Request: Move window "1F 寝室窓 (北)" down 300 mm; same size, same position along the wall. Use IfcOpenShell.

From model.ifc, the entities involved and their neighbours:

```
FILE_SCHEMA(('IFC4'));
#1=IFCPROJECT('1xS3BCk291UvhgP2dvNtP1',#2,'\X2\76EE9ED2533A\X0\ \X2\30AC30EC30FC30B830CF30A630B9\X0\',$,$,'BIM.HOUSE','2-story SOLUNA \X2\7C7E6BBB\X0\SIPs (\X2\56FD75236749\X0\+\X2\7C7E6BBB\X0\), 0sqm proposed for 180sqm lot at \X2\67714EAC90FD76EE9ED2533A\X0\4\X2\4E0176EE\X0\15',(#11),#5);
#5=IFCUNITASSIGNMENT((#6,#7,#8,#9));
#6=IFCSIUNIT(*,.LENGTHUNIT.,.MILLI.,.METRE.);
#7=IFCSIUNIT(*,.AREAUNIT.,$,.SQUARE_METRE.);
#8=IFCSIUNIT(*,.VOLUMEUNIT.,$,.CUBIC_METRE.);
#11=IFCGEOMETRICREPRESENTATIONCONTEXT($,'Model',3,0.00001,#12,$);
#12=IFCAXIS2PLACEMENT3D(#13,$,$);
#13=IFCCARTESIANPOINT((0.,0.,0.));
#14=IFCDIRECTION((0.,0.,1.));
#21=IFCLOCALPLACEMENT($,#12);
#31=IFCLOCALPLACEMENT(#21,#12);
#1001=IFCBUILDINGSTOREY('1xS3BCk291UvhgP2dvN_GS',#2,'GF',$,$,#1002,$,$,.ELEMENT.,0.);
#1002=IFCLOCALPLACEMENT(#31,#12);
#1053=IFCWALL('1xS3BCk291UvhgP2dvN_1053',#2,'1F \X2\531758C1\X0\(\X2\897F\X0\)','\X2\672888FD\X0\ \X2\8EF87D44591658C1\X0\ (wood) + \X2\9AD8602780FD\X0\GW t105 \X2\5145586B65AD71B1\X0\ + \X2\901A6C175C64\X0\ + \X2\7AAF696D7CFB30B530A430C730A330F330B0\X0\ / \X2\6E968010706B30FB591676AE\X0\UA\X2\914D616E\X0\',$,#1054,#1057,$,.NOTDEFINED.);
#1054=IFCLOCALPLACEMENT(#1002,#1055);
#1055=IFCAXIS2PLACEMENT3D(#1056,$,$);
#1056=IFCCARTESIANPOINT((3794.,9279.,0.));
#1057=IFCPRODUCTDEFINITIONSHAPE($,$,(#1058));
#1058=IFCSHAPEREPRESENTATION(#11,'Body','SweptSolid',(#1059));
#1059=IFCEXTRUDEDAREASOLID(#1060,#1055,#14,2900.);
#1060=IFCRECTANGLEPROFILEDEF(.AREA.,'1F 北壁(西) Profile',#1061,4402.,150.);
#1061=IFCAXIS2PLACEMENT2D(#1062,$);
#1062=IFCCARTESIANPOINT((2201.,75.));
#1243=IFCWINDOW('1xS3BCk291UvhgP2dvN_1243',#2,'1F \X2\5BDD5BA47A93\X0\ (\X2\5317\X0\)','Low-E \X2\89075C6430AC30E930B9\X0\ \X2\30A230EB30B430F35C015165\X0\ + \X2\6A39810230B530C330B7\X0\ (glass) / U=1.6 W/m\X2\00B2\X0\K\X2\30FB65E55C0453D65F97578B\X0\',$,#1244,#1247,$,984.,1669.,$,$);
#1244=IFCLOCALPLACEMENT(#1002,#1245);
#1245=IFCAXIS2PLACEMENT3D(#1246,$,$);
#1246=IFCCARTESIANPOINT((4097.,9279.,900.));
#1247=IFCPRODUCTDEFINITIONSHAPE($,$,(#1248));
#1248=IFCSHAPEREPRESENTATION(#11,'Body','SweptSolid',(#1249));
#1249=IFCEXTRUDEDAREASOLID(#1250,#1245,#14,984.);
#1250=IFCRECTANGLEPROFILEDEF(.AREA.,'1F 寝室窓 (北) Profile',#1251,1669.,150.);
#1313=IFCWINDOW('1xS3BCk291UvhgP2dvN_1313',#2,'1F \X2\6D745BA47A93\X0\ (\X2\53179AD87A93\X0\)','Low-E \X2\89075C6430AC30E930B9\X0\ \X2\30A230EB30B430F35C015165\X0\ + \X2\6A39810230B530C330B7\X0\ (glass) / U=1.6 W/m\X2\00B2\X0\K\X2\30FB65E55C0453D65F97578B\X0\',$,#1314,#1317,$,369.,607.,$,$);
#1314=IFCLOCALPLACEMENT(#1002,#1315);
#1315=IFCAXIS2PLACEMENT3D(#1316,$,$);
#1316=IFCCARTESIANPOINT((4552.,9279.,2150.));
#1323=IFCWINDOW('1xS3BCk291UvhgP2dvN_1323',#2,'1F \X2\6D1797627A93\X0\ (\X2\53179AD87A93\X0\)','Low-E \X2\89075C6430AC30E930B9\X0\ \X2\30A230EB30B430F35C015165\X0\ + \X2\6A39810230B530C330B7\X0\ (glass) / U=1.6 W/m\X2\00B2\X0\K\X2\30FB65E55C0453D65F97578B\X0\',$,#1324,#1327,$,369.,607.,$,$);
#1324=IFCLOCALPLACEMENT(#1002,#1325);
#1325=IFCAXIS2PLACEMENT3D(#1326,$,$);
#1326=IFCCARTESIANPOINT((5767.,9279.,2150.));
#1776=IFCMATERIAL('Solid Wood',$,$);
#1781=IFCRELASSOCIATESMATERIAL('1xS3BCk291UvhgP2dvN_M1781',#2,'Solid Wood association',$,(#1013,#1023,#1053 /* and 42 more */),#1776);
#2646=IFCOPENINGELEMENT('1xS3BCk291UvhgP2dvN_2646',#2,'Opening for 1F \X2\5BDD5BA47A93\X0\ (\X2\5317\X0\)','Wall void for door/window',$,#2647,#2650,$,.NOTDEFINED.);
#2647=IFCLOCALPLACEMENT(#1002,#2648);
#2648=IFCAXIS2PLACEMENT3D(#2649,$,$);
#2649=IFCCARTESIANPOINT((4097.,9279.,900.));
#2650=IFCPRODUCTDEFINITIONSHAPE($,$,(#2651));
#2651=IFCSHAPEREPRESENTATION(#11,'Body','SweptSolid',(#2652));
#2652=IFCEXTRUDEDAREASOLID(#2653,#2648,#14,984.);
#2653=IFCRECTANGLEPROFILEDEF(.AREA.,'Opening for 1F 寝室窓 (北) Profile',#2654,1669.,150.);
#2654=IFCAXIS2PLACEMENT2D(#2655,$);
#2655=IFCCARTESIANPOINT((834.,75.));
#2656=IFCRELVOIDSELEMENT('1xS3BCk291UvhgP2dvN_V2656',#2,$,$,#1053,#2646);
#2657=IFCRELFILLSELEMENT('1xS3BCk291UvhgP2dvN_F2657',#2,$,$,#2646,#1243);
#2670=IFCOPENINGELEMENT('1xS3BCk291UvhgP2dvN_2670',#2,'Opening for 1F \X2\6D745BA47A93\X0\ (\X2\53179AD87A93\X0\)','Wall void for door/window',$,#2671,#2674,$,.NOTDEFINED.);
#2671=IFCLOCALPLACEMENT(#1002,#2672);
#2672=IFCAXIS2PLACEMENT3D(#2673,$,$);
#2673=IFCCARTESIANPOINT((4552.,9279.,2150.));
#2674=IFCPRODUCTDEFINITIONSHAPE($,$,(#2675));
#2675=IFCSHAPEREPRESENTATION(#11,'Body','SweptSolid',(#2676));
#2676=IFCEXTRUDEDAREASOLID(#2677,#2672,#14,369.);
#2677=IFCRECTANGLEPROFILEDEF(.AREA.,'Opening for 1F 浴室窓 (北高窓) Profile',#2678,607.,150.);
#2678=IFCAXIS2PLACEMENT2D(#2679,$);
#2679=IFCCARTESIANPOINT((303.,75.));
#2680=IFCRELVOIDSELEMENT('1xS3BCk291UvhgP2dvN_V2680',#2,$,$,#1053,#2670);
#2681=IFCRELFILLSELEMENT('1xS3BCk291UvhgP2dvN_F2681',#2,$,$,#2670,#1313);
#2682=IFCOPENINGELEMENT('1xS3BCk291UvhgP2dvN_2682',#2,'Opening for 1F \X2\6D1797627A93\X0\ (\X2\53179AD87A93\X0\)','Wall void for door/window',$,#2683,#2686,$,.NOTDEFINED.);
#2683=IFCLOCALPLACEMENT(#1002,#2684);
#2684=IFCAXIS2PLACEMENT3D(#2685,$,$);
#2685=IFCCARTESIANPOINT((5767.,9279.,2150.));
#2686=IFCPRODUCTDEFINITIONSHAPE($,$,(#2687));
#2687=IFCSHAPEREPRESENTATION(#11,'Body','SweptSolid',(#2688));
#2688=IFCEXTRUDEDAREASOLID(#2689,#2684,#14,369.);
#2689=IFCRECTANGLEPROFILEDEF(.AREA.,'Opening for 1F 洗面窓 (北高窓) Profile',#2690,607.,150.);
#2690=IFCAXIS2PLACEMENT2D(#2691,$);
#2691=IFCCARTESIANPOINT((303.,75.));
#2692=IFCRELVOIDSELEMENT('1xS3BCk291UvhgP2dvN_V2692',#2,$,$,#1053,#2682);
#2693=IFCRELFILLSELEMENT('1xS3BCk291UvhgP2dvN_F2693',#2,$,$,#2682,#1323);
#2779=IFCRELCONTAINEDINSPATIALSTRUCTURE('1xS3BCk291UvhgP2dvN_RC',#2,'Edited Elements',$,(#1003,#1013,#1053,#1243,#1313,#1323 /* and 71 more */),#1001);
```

```python
import numpy as np
import ifcopenshell
import ifcopenshell.api.geometry
import ifcopenshell.util.placement
import ifcopenshell.util.unit

model = ifcopenshell.open("model.ifc")
unit_scale = ifcopenshell.util.unit.calculate_unit_scale(model)

window = model.by_id(1243)
opening = window.FillsVoids[0].RelatingOpeningElement
dz = -0.3 / unit_scale

shift = np.array([0.0, 0.0, dz])
# The window is not placed relative to its opening, so move both.
for product in (opening, window):
    matrix = ifcopenshell.util.placement.get_local_placement(product.ObjectPlacement)
    matrix[:3, 3] += shift
    ifcopenshell.api.geometry.edit_object_placement(model, product=product, matrix=matrix, is_si=False)

print(f"moved by {dz * unit_scale:+.3f} m")

model.write("model_updated.ifc")
```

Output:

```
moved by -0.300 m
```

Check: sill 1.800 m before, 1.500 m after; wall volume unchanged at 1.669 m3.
